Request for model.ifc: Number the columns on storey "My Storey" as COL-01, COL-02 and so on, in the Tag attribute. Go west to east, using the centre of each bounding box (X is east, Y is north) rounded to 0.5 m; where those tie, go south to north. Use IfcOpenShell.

First a look at what the model holds.

```python
import ifcopenshell
import ifcopenshell.util.element
import ifcopenshell.util.placement

model = ifcopenshell.open("model.ifc")
print(model.schema)
storey = next(s for s in model.by_type("IfcBuildingStorey") if s.Name == "My Storey")
columns = [e for e in ifcopenshell.util.element.get_decomposition(storey) if e.is_a("IfcColumn")]
for e in sorted(columns, key=lambda e: e.id()):
    origin = ifcopenshell.util.placement.get_local_placement(e.ObjectPlacement)[:3, 3]
    print(e.id(), e.Tag, e.Name, origin.round(2) + 0.0, sep=" | ")
```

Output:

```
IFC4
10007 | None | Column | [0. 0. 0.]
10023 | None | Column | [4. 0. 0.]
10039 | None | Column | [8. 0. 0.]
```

```python
import ifcopenshell
import ifcopenshell.geom
import ifcopenshell.util.element
import ifcopenshell.util.shape

model = ifcopenshell.open("model.ifc")
settings = ifcopenshell.geom.settings()
settings.set("use-world-coords", True)


def centre(element):
    shape = ifcopenshell.geom.create_shape(settings, element)
    return ifcopenshell.util.shape.get_bbox_centroid(shape.geometry)


storey = next(s for s in model.by_type("IfcBuildingStorey") if s.Name == "My Storey")
columns = [e for e in ifcopenshell.util.element.get_decomposition(storey) if e.is_a("IfcColumn")]

# Insertion points can sit at a corner or the storey origin, so sort by the geometry (in metres).
centres = {e: centre(e) for e in columns}
columns.sort(key=lambda e: (round(centres[e][0] / 0.5), centres[e][1]))

for i, e in enumerate(columns, start=1):
    number = f"COL-{i:02d}"
    e.Tag = number
    print(e.id(), number)

model.write("model_v2.ifc")
```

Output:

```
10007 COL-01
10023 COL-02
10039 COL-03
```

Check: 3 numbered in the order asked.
